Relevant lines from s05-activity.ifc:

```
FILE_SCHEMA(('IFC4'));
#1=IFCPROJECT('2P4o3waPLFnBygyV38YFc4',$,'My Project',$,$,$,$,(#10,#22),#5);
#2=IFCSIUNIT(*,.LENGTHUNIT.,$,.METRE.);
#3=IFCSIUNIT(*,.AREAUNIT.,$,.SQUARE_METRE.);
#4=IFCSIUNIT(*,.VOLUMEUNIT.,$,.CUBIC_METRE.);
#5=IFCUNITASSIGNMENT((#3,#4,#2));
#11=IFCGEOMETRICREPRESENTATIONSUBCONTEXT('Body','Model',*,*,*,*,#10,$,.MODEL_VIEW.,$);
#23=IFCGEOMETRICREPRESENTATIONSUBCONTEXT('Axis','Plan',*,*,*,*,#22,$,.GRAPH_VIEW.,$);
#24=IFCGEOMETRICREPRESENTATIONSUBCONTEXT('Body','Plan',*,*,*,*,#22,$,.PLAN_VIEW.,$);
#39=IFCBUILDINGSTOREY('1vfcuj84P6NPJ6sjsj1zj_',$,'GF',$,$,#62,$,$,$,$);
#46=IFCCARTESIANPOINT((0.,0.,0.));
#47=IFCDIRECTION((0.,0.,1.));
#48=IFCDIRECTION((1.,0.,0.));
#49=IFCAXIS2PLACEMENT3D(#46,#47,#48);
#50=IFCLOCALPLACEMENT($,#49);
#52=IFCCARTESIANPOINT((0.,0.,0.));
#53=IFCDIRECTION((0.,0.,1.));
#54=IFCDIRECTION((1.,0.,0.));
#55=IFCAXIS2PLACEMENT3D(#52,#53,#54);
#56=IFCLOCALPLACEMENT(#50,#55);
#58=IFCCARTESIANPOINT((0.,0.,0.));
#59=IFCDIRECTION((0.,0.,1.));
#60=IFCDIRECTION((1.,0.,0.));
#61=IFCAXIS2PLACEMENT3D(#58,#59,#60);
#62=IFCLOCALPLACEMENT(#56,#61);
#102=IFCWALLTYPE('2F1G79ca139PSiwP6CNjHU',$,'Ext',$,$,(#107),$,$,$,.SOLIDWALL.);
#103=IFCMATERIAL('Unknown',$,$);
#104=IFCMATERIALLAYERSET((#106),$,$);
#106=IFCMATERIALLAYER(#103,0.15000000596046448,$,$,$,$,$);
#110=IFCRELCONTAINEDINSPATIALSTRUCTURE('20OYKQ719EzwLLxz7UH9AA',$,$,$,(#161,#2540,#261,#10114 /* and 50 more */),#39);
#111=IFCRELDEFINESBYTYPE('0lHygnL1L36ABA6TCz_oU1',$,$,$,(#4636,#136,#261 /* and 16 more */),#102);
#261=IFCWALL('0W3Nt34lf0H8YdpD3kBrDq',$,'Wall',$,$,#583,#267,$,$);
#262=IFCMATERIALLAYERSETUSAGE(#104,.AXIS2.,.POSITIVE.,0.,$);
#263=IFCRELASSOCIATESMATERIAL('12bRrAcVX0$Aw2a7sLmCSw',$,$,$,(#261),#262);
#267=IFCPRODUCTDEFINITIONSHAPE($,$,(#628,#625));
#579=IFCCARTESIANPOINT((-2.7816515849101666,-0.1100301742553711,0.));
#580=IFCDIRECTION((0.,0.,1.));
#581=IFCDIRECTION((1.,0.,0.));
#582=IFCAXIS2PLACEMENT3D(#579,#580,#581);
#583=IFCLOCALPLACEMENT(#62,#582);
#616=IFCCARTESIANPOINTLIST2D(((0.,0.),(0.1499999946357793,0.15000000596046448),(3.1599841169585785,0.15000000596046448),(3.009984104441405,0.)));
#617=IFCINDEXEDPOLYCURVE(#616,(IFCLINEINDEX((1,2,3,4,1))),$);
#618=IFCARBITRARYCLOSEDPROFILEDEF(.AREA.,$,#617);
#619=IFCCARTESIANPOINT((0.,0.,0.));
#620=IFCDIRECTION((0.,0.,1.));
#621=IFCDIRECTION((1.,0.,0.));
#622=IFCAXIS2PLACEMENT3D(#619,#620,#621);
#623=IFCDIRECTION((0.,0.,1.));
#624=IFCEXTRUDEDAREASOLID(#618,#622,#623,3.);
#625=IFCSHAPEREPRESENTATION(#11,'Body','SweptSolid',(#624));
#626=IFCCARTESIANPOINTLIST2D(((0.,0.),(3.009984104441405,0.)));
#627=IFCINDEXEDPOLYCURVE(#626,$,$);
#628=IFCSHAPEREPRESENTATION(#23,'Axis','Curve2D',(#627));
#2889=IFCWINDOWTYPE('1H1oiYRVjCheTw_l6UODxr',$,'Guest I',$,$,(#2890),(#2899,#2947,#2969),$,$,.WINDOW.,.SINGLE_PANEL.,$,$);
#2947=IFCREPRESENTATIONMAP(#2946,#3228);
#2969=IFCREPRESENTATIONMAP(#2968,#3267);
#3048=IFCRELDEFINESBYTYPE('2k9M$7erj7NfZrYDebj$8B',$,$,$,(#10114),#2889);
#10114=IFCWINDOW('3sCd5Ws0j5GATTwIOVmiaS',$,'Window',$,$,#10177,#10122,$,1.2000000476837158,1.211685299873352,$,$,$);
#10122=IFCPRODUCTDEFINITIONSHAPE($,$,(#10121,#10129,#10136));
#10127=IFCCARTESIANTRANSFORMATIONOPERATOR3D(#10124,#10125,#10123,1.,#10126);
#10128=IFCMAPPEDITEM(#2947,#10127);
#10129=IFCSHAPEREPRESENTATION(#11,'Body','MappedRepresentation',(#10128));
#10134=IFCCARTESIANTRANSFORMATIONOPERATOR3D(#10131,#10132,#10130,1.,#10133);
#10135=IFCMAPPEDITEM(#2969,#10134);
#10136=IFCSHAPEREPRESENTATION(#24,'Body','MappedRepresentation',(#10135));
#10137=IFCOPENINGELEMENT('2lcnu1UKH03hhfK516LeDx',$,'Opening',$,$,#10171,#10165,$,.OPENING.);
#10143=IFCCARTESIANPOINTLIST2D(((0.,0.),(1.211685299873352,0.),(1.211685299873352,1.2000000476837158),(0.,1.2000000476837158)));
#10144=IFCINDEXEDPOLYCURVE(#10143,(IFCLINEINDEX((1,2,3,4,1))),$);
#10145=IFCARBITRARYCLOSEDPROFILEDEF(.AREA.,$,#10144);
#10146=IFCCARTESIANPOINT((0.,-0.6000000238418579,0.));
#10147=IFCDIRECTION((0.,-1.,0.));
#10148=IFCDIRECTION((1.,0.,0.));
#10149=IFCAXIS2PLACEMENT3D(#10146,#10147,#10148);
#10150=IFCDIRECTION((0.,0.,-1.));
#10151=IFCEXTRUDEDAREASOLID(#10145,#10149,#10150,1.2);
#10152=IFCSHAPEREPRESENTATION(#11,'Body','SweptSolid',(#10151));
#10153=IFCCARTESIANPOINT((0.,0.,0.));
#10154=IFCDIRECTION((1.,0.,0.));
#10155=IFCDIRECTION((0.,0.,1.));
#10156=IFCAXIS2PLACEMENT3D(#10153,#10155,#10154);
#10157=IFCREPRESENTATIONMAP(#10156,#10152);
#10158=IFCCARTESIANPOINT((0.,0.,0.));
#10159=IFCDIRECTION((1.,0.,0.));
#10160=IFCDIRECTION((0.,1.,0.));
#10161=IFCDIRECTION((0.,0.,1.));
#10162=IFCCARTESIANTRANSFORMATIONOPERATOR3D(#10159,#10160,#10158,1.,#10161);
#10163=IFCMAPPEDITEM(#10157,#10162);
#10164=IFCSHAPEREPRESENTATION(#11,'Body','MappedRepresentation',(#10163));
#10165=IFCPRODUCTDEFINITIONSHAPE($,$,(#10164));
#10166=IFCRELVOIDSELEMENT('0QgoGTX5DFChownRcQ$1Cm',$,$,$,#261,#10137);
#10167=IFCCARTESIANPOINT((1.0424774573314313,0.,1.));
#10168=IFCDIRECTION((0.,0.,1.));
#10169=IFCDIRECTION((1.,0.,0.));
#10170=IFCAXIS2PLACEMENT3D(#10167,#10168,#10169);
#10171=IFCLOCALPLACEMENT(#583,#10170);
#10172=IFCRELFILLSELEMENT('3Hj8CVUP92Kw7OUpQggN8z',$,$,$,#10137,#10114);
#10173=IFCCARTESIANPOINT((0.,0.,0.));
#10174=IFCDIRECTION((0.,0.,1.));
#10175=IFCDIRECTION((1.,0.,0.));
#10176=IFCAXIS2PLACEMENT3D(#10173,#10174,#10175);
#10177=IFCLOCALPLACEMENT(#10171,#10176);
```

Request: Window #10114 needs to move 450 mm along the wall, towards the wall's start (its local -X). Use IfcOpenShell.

```python
import ifcopenshell
import ifcopenshell.api.geometry
import ifcopenshell.util.placement
import ifcopenshell.util.unit

model = ifcopenshell.open("s05-activity.ifc")
unit_scale = ifcopenshell.util.unit.calculate_unit_scale(model)

window = model.by_guid("3sCd5Ws0j5GATTwIOVmiaS")
opening = window.FillsVoids[0].RelatingOpeningElement
wall = opening.VoidsElements[0].RelatingBuildingElement

wall_matrix = ifcopenshell.util.placement.get_local_placement(wall.ObjectPlacement)
shift = wall_matrix[:3, 0] * -0.45 / unit_scale
before = ifcopenshell.util.placement.get_local_placement(window.ObjectPlacement)[:3, 3].copy()

# The window is placed relative to its opening, so it follows when the opening moves.
matrix = ifcopenshell.util.placement.get_local_placement(opening.ObjectPlacement)
matrix[:3, 3] += shift
ifcopenshell.api.geometry.edit_object_placement(
    model, product=opening, matrix=matrix, is_si=False, should_transform_children=True
)

after = ifcopenshell.util.placement.get_local_placement(window.ObjectPlacement)[:3, 3]
print("window moved by", (after - before).round(3) + 0.0)

model.write("s05-activity-out.ifc")
```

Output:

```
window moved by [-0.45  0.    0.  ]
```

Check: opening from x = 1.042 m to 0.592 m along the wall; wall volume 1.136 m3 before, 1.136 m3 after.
